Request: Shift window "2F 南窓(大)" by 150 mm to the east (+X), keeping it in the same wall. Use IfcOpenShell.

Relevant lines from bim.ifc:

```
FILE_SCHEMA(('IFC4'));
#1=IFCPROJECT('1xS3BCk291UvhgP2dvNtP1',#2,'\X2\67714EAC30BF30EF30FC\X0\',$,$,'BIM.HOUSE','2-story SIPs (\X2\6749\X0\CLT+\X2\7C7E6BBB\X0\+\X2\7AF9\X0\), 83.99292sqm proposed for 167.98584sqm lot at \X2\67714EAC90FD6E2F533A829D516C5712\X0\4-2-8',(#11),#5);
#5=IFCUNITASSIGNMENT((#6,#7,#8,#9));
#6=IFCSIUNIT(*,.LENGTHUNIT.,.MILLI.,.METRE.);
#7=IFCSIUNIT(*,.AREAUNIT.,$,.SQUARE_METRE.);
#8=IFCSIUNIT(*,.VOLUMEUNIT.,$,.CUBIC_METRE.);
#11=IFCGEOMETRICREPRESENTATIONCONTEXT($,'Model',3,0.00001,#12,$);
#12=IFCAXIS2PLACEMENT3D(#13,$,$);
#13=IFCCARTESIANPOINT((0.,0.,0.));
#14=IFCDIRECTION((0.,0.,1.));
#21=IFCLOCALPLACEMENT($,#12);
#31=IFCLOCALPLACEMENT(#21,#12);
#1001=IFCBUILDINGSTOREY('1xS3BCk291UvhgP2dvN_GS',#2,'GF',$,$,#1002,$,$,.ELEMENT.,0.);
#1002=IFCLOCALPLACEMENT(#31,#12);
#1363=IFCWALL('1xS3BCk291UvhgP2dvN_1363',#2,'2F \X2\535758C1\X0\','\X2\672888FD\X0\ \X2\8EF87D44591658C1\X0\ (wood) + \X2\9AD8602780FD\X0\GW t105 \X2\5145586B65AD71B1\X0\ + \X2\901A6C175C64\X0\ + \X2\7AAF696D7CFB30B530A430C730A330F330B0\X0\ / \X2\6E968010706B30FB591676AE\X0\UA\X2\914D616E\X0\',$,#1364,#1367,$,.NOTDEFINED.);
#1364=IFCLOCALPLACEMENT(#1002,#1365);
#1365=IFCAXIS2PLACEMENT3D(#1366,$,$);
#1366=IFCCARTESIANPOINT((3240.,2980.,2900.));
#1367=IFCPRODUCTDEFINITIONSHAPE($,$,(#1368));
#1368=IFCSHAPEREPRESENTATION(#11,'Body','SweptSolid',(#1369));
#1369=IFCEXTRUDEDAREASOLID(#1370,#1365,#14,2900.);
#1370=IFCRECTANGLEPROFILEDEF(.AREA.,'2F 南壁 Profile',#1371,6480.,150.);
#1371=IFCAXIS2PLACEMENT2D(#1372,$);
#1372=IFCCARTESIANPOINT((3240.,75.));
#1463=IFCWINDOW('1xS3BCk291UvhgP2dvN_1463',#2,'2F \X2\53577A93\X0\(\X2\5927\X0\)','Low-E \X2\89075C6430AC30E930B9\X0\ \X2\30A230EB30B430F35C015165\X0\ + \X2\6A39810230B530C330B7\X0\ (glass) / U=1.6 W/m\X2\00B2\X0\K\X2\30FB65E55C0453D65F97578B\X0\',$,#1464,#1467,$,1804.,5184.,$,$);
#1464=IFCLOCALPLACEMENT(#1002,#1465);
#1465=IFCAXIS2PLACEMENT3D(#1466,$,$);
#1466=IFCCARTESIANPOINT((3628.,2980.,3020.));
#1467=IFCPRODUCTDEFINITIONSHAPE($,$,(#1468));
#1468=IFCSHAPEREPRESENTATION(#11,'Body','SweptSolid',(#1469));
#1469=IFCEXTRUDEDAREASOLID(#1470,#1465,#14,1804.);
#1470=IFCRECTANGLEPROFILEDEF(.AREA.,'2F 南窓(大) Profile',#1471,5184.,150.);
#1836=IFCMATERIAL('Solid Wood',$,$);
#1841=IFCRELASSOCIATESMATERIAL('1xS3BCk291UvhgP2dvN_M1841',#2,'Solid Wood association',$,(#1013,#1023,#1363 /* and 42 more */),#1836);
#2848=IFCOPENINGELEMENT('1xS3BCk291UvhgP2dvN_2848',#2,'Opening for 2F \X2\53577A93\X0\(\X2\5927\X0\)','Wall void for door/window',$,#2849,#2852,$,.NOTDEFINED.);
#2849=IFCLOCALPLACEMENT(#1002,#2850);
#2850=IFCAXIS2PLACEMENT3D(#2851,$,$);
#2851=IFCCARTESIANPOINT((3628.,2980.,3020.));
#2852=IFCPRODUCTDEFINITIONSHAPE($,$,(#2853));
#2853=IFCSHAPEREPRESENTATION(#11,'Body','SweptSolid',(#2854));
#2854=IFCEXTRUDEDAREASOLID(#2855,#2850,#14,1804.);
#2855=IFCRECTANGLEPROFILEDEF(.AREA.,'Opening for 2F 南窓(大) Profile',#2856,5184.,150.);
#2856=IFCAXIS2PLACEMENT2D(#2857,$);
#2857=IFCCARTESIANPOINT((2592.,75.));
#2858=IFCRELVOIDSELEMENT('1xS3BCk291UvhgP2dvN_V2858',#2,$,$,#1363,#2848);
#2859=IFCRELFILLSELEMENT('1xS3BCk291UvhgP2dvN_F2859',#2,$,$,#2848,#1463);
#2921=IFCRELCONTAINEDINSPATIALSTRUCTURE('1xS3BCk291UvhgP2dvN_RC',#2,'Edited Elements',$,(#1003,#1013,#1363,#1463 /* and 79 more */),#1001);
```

```python
import ifcopenshell
import ifcopenshell.api.geometry
import ifcopenshell.util.placement
import ifcopenshell.util.unit

model = ifcopenshell.open("bim.ifc")
unit_scale = ifcopenshell.util.unit.calculate_unit_scale(model)

window = model.by_guid("1xS3BCk291UvhgP2dvN_1463")
opening = window.FillsVoids[0].RelatingOpeningElement
wall = opening.VoidsElements[0].RelatingBuildingElement

wall_matrix = ifcopenshell.util.placement.get_local_placement(wall.ObjectPlacement)
shift = wall_matrix[:3, 0] * 0.15 / unit_scale
before = ifcopenshell.util.placement.get_local_placement(window.ObjectPlacement)[:3, 3].copy()

# The window is not placed relative to its opening, so move both.
for product in (opening, window):
    matrix = ifcopenshell.util.placement.get_local_placement(product.ObjectPlacement)
    matrix[:3, 3] += shift
    ifcopenshell.api.geometry.edit_object_placement(model, product=product, matrix=matrix, is_si=False)

after = ifcopenshell.util.placement.get_local_placement(window.ObjectPlacement)[:3, 3]
print("window moved by", (after - before).round(3) + 0.0)

model.write("bim_v2.ifc")
```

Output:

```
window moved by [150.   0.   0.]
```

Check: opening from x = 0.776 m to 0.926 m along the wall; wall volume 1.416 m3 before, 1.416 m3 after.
